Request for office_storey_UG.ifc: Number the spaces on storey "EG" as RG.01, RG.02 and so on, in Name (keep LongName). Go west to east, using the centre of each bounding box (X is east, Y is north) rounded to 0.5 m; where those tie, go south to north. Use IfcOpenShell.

First a look at what the model holds.

```python
import ifcopenshell
import ifcopenshell.util.element
import ifcopenshell.util.placement

model = ifcopenshell.open("office_storey_UG.ifc")
print(model.schema)
storey = next(s for s in model.by_type("IfcBuildingStorey") if s.Name == "EG")
spaces = [e for e in ifcopenshell.util.element.get_decomposition(storey) if e.is_a("IfcSpace")]
for e in sorted(spaces, key=lambda e: e.id()):
    origin = ifcopenshell.util.placement.get_local_placement(e.ObjectPlacement)[:3, 3]
    print(e.id(), e.Name, e.LongName, origin.round(2) + 0.0, sep=" | ")
```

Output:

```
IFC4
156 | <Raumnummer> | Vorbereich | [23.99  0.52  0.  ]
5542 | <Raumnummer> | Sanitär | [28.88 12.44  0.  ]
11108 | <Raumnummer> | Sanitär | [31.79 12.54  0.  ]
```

```python
import ifcopenshell
import ifcopenshell.geom
import ifcopenshell.util.element
import ifcopenshell.util.shape

model = ifcopenshell.open("office_storey_UG.ifc")
settings = ifcopenshell.geom.settings()
settings.set("use-world-coords", True)


def centre(element):
    shape = ifcopenshell.geom.create_shape(settings, element)
    return ifcopenshell.util.shape.get_bbox_centroid(shape.geometry)


storey = next(s for s in model.by_type("IfcBuildingStorey") if s.Name == "EG")
spaces = [e for e in ifcopenshell.util.element.get_decomposition(storey) if e.is_a("IfcSpace")]

# Insertion points can sit at a corner or the storey origin, so sort by the geometry (in metres).
centres = {e: centre(e) for e in spaces}
spaces.sort(key=lambda e: (round(centres[e][0] / 0.5), centres[e][1]))

for i, e in enumerate(spaces, start=1):
    number = f"RG.{i:02d}"
    e.Name = number
    print(e.id(), number)

model.write("office_storey_UG-out.ifc")
```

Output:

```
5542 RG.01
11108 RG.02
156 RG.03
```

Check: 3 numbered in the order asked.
